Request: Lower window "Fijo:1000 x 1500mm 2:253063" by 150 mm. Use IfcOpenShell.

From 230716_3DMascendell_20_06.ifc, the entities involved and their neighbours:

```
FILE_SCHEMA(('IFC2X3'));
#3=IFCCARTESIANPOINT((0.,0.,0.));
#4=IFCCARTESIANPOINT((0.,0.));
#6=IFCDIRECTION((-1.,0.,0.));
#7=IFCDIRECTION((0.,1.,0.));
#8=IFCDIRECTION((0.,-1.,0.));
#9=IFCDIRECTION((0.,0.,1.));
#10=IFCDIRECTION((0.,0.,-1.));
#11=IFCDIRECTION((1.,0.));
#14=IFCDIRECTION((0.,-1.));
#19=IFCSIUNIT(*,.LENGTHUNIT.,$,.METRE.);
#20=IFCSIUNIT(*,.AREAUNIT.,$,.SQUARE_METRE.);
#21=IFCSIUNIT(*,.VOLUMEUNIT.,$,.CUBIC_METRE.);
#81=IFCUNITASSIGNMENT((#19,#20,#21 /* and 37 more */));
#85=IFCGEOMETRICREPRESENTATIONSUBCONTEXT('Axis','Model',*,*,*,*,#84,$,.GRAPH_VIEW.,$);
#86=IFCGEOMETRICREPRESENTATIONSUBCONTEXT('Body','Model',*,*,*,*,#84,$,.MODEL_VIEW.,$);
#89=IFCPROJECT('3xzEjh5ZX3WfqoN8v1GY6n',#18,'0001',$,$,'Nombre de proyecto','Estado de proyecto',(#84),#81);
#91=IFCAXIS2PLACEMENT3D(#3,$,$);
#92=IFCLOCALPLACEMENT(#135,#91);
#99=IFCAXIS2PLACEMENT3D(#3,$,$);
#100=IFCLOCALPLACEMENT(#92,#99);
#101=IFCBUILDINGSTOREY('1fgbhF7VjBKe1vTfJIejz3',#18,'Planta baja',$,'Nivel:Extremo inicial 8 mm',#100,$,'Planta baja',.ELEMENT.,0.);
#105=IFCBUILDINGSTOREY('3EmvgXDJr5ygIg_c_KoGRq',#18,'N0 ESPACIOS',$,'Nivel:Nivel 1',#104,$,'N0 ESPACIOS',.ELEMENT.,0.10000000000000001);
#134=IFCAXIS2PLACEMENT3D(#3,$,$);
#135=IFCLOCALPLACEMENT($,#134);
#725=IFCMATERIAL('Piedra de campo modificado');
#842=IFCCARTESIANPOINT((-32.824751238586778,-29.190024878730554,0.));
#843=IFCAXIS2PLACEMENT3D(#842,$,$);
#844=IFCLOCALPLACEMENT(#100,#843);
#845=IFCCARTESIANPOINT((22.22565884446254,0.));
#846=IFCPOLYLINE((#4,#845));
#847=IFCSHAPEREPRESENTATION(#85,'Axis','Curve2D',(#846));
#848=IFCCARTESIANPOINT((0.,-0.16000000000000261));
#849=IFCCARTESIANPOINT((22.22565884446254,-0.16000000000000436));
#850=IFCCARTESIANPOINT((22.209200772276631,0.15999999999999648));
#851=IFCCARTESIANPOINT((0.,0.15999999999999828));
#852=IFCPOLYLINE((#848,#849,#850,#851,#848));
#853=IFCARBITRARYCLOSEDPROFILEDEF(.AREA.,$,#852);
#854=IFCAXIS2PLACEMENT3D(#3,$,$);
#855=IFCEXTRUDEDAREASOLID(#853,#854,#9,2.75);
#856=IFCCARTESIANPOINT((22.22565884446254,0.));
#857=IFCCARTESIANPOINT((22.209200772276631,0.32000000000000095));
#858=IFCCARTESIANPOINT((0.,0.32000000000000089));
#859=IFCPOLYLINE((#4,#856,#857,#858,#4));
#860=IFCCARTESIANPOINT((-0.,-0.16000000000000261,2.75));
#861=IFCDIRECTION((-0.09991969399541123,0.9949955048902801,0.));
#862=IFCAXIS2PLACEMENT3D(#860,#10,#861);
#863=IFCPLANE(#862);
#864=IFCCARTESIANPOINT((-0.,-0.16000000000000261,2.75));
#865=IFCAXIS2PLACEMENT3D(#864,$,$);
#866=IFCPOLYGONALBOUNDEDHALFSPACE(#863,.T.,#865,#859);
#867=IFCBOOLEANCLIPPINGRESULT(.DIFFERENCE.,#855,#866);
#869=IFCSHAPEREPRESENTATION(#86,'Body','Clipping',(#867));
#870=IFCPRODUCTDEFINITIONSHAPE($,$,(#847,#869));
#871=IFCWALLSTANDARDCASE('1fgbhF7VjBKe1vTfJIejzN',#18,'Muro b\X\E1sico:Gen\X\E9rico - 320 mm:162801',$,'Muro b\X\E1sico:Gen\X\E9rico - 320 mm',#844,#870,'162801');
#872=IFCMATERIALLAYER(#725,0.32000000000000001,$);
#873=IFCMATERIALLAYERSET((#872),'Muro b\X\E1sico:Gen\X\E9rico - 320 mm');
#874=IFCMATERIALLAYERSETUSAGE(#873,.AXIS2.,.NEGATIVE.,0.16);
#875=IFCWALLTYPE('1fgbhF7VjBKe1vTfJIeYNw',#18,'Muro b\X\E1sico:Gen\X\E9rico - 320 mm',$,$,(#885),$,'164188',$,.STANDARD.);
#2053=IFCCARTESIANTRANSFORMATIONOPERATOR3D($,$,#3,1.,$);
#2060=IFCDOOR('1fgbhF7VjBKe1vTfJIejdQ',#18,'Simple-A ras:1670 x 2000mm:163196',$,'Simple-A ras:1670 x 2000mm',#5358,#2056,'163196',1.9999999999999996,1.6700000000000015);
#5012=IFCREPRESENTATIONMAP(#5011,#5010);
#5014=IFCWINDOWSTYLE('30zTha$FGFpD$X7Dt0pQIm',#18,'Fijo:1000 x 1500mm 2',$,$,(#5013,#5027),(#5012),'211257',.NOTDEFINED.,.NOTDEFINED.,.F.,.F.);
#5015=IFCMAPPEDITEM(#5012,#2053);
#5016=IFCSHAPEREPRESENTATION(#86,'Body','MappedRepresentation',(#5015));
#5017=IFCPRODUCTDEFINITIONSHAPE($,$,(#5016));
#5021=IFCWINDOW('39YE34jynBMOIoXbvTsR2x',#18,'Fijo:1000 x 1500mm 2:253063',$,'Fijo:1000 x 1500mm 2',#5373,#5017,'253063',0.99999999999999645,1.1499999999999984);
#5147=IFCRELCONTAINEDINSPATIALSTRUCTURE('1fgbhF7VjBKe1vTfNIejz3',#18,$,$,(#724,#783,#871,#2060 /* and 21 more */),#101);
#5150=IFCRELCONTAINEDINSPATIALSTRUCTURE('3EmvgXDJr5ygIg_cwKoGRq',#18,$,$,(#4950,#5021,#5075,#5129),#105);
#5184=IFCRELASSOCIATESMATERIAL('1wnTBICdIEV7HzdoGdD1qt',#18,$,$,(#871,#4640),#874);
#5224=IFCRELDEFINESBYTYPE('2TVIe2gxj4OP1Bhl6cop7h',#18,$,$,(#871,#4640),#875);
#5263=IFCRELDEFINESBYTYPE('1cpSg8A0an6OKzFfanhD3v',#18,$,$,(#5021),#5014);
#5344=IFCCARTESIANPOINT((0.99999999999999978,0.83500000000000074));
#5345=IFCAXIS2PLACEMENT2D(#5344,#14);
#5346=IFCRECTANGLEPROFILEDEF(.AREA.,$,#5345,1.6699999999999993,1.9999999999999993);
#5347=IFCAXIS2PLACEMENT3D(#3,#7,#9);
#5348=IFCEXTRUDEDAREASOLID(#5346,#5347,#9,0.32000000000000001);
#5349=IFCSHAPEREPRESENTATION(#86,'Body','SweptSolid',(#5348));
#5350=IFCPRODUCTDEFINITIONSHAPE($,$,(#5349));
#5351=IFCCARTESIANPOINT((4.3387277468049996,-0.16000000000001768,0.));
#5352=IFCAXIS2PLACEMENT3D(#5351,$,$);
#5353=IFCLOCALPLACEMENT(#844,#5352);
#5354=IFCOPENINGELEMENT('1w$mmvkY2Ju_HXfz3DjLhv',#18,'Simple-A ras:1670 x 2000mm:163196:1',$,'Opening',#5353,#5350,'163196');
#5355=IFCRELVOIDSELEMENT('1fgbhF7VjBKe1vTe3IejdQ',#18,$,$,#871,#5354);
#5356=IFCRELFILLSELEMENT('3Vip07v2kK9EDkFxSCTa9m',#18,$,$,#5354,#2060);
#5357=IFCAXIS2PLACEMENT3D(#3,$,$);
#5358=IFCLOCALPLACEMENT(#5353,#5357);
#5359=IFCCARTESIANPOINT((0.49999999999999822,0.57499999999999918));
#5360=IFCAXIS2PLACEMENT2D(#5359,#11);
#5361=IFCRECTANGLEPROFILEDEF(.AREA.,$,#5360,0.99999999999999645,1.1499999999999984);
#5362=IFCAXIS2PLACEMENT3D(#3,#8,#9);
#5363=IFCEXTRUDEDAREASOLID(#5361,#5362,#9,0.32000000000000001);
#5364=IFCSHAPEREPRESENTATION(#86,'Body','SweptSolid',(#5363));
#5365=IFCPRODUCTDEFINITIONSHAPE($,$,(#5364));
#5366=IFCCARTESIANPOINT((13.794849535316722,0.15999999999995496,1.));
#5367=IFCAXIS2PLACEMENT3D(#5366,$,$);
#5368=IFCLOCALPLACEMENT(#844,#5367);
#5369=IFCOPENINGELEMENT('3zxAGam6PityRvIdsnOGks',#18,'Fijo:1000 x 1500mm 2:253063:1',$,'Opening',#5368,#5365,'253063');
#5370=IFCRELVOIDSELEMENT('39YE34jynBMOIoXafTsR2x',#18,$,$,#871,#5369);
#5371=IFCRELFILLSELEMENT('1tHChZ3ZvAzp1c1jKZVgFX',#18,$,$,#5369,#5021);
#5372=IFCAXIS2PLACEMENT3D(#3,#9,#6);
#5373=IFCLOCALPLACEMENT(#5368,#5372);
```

```python
import numpy as np
import ifcopenshell
import ifcopenshell.api.geometry
import ifcopenshell.util.placement
import ifcopenshell.util.unit

model = ifcopenshell.open("230716_3DMascendell_20_06.ifc")
unit_scale = ifcopenshell.util.unit.calculate_unit_scale(model)

window = model.by_id(5021)
opening = window.FillsVoids[0].RelatingOpeningElement
dz = -0.15

shift = np.array([0.0, 0.0, dz])
# The window is placed relative to its opening, so it follows when the opening moves.
matrix = ifcopenshell.util.placement.get_local_placement(opening.ObjectPlacement)
matrix[:3, 3] += shift
ifcopenshell.api.geometry.edit_object_placement(
    model, product=opening, matrix=matrix, is_si=False, should_transform_children=True
)

print(f"moved by {dz * unit_scale:+.3f} m")

model.write("230716_3DMascendell_20_06_rev.ifc")
```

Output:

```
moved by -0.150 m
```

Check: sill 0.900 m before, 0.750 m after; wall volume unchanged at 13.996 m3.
